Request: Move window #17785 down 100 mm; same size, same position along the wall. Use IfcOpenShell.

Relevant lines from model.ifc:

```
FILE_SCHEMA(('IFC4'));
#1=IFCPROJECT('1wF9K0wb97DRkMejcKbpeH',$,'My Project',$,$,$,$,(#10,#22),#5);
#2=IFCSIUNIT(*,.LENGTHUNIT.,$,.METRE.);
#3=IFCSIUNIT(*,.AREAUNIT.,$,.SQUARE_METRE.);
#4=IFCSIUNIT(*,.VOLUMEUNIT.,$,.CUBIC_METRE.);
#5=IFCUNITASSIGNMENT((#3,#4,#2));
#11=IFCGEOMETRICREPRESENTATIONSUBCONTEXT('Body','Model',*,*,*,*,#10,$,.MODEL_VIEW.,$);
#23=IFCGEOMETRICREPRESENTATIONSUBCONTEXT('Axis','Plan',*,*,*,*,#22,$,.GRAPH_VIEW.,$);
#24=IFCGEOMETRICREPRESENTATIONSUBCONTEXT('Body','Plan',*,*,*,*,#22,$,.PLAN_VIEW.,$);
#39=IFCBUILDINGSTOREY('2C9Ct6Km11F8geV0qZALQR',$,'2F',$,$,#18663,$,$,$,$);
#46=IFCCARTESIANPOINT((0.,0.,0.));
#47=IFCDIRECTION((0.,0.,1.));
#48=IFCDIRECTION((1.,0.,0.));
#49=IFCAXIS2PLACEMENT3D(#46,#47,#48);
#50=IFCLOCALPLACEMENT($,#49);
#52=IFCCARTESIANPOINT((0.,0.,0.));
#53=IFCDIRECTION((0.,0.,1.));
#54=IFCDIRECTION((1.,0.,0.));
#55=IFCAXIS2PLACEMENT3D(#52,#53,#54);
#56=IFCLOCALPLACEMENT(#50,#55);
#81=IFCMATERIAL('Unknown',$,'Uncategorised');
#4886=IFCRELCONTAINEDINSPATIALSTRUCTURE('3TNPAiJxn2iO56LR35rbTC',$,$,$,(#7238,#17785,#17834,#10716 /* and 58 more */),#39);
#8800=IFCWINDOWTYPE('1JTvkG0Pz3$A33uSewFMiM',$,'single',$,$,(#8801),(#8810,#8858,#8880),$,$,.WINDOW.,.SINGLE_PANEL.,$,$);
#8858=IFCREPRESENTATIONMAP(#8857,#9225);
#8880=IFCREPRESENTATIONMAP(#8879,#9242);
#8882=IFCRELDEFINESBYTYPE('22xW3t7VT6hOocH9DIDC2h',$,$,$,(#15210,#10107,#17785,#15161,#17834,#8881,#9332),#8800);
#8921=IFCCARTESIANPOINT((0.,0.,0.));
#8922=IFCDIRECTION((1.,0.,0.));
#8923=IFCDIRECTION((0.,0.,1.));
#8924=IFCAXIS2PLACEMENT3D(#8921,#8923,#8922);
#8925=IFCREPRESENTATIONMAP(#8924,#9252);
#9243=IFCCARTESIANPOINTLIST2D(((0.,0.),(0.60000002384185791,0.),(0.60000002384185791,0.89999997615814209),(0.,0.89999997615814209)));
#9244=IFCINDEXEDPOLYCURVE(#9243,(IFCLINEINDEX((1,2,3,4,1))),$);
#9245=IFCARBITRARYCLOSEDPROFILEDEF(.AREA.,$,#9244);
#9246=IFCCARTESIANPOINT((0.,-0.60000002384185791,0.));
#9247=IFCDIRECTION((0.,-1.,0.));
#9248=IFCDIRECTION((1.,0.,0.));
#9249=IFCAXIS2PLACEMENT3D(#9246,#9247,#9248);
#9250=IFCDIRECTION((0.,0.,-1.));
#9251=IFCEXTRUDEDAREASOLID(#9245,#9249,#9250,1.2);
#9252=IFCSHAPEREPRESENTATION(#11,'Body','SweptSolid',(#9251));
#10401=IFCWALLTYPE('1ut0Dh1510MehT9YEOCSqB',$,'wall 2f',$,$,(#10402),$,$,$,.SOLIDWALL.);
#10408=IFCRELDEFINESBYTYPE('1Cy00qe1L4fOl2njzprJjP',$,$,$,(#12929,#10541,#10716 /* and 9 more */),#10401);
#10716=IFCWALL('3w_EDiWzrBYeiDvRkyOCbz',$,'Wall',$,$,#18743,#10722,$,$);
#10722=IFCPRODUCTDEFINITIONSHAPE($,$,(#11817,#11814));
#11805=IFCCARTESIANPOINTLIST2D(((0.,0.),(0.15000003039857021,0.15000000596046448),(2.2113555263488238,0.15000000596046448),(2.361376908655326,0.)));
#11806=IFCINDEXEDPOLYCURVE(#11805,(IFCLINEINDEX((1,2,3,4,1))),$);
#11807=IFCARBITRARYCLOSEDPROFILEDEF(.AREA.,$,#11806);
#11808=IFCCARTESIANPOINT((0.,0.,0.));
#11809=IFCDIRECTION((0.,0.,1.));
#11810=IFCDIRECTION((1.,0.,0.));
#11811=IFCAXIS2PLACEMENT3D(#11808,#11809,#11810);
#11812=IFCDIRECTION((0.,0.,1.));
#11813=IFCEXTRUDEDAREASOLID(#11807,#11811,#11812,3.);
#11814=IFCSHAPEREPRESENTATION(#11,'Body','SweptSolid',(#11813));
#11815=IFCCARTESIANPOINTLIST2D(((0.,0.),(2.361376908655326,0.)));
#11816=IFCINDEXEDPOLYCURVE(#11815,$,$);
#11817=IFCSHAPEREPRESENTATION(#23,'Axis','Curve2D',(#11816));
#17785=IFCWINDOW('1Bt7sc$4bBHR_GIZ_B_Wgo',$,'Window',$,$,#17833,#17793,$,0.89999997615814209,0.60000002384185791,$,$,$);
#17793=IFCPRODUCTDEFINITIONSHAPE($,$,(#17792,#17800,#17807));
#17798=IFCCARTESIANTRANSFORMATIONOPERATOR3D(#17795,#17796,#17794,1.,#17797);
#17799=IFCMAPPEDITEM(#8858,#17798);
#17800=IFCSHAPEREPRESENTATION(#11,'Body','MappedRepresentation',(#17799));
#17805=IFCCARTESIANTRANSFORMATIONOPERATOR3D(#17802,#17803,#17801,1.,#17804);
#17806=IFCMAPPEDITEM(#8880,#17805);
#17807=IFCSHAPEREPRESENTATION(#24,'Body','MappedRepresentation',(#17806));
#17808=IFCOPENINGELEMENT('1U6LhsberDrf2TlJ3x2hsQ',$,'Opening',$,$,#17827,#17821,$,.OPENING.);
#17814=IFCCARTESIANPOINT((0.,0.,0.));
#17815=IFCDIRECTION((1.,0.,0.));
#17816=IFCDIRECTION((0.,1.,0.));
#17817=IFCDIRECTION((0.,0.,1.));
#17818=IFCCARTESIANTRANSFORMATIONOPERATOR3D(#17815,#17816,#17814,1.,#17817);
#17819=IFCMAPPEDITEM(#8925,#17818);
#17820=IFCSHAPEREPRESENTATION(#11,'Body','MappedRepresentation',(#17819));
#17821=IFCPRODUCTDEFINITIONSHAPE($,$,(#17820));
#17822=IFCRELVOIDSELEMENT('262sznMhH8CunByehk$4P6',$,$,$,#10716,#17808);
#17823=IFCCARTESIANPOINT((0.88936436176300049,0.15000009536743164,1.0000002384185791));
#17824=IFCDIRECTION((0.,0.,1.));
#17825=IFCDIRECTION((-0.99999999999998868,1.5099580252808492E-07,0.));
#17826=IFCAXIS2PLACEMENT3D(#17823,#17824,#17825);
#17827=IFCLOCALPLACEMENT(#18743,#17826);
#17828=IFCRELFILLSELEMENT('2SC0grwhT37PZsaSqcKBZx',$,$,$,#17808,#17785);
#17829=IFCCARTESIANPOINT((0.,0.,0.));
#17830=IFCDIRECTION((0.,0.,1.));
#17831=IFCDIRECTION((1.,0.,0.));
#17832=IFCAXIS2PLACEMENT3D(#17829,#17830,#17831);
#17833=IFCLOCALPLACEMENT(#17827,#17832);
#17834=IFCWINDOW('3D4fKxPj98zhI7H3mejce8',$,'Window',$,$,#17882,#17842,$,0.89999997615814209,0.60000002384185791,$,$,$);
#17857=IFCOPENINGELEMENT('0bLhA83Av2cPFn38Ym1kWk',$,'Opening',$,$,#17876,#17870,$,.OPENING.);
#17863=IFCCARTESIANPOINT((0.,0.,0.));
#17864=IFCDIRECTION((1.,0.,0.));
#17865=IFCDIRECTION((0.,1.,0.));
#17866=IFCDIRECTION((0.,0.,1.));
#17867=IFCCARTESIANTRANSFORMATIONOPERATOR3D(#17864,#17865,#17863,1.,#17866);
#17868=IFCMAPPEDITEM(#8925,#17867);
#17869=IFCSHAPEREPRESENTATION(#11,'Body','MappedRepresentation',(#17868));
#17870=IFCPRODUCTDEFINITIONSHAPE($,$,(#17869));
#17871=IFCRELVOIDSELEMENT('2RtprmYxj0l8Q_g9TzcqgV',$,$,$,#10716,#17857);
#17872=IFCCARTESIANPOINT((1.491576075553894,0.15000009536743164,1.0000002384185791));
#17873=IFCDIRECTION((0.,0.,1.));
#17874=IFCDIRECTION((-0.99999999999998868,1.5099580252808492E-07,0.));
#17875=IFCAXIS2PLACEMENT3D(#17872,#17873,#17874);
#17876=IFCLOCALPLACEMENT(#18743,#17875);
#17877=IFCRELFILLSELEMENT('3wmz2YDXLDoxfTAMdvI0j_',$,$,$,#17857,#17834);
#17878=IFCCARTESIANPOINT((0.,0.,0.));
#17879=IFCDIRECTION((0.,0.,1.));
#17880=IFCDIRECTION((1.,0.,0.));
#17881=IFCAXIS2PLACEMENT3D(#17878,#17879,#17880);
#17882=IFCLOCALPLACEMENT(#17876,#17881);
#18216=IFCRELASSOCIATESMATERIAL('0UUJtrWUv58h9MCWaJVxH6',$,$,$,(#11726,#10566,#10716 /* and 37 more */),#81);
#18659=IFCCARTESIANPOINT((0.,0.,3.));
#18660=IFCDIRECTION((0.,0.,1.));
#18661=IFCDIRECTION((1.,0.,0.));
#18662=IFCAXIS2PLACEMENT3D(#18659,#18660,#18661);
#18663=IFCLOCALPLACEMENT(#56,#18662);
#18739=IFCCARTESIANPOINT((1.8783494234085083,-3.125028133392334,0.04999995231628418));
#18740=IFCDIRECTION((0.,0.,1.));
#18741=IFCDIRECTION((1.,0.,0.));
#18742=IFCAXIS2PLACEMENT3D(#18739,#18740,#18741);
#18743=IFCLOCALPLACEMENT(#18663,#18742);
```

```python
import numpy as np
import ifcopenshell
import ifcopenshell.api.geometry
import ifcopenshell.util.placement
import ifcopenshell.util.unit

model = ifcopenshell.open("model.ifc")
unit_scale = ifcopenshell.util.unit.calculate_unit_scale(model)

window = model.by_id(17785)
opening = window.FillsVoids[0].RelatingOpeningElement
dz = -0.1

shift = np.array([0.0, 0.0, dz])
# The window is placed relative to its opening, so it follows when the opening moves.
matrix = ifcopenshell.util.placement.get_local_placement(opening.ObjectPlacement)
matrix[:3, 3] += shift
ifcopenshell.api.geometry.edit_object_placement(
    model, product=opening, matrix=matrix, is_si=False, should_transform_children=True
)

print(f"moved by {dz * unit_scale:+.3f} m")

model.write("model_rev.ifc")
```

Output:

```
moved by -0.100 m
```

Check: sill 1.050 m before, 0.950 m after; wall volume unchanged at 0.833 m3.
